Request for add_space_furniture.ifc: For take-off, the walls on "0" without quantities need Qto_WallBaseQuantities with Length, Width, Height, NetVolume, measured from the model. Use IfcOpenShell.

First a look at what the model holds.

```python
import ifcopenshell
import ifcopenshell.util.element
import ifcopenshell.util.unit

model = ifcopenshell.open("add_space_furniture.ifc")
print(model.schema)
for unit_type in ("LENGTHUNIT", "AREAUNIT", "VOLUMEUNIT"):
    print(unit_type, ifcopenshell.util.unit.calculate_unit_scale(model, unit_type))
storey = next(s for s in model.by_type("IfcBuildingStorey") if s.Name == "0")
walls = [e for e in ifcopenshell.util.element.get_decomposition(storey) if e.is_a("IfcWall")]
for e in sorted(walls, key=lambda e: e.id()):
    print(e.id(), e.is_a(), e.Name, list(ifcopenshell.util.element.get_psets(e, qtos_only=True)), sep=" | ")
```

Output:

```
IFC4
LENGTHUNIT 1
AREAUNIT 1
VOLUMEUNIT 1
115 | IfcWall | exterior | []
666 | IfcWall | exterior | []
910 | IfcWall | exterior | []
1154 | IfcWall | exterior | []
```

```python
import ifcopenshell
import ifcopenshell.api.pset
import ifcopenshell.geom
import ifcopenshell.util.element
import ifcopenshell.util.shape
import ifcopenshell.util.unit

model = ifcopenshell.open("add_space_furniture.ifc")
unit_scale = ifcopenshell.util.unit.calculate_unit_scale(model)
volume_scale = ifcopenshell.util.unit.calculate_unit_scale(model, "VOLUMEUNIT")
settings = ifcopenshell.geom.settings()

storey = next(s for s in model.by_type("IfcBuildingStorey") if s.Name == "0")
walls = [e for e in ifcopenshell.util.element.get_decomposition(storey) if e.is_a("IfcWall")]

for e in sorted(walls, key=lambda e: e.id()):
    if ifcopenshell.util.element.get_psets(e, qtos_only=True, should_inherit=False):
        continue
    # Geometry comes back in metres, in the element's own axes.
    shape = ifcopenshell.geom.create_shape(settings, e)
    values = {
        "Length": ifcopenshell.util.shape.get_x(shape.geometry) / unit_scale,
        "Width": ifcopenshell.util.shape.get_y(shape.geometry) / unit_scale,
        "Height": ifcopenshell.util.shape.get_z(shape.geometry) / unit_scale,
        "NetVolume": ifcopenshell.util.shape.get_volume(shape.geometry) / volume_scale,
    }
    qto = ifcopenshell.api.pset.add_qto(model, product=e, name="Qto_WallBaseQuantities")
    ifcopenshell.api.pset.edit_qto(model, qto=qto, properties=values)
    print(e.id(), {k: round(v, 3) for k, v in values.items()})

model.write("add_space_furniture_edited.ifc")
```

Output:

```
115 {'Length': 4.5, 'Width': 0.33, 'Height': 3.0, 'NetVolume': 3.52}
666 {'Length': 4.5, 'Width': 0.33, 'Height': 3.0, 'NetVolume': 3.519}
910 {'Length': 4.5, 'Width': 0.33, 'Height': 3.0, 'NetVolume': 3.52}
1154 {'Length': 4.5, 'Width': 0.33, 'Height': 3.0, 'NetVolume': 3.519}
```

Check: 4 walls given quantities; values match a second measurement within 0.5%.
